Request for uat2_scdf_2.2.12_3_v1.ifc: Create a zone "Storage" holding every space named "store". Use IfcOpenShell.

First a look at what the model holds.

```python
import ifcopenshell

model = ifcopenshell.open("uat2_scdf_2.2.12_3_v1.ifc")
print(model.schema)
seen = {}
for space in model.by_type("IfcSpace"):
    seen[space.LongName] = seen.get(space.LongName, 0) + 1
for name, count in sorted(seen.items(), key=str):
    print(count, "x", name)
print("zones:", [z.Name for z in model.by_type("IfcZone")][:20])
```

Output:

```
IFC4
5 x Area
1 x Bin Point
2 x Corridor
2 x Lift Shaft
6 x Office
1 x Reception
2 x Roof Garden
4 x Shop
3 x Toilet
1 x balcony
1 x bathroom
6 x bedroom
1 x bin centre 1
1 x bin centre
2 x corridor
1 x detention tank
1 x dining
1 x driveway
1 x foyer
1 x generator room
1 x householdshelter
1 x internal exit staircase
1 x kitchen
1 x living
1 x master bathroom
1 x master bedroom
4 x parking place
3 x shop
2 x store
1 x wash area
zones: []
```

```python
import ifcopenshell
import ifcopenshell.api.group
import ifcopenshell.api.root

model = ifcopenshell.open("uat2_scdf_2.2.12_3_v1.ifc")

names = {"store"}
spaces = [s for s in model.by_type("IfcSpace") if s.LongName in names]

zone = ifcopenshell.api.root.create_entity(model, ifc_class="IfcZone", name="Storage")
ifcopenshell.api.group.assign_group(model, products=spaces, group=zone)
print(len(spaces), "spaces in", zone.Name)

model.write("uat2_scdf_2.2.12_3_v1_v2.ifc")
```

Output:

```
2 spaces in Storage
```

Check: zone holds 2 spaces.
